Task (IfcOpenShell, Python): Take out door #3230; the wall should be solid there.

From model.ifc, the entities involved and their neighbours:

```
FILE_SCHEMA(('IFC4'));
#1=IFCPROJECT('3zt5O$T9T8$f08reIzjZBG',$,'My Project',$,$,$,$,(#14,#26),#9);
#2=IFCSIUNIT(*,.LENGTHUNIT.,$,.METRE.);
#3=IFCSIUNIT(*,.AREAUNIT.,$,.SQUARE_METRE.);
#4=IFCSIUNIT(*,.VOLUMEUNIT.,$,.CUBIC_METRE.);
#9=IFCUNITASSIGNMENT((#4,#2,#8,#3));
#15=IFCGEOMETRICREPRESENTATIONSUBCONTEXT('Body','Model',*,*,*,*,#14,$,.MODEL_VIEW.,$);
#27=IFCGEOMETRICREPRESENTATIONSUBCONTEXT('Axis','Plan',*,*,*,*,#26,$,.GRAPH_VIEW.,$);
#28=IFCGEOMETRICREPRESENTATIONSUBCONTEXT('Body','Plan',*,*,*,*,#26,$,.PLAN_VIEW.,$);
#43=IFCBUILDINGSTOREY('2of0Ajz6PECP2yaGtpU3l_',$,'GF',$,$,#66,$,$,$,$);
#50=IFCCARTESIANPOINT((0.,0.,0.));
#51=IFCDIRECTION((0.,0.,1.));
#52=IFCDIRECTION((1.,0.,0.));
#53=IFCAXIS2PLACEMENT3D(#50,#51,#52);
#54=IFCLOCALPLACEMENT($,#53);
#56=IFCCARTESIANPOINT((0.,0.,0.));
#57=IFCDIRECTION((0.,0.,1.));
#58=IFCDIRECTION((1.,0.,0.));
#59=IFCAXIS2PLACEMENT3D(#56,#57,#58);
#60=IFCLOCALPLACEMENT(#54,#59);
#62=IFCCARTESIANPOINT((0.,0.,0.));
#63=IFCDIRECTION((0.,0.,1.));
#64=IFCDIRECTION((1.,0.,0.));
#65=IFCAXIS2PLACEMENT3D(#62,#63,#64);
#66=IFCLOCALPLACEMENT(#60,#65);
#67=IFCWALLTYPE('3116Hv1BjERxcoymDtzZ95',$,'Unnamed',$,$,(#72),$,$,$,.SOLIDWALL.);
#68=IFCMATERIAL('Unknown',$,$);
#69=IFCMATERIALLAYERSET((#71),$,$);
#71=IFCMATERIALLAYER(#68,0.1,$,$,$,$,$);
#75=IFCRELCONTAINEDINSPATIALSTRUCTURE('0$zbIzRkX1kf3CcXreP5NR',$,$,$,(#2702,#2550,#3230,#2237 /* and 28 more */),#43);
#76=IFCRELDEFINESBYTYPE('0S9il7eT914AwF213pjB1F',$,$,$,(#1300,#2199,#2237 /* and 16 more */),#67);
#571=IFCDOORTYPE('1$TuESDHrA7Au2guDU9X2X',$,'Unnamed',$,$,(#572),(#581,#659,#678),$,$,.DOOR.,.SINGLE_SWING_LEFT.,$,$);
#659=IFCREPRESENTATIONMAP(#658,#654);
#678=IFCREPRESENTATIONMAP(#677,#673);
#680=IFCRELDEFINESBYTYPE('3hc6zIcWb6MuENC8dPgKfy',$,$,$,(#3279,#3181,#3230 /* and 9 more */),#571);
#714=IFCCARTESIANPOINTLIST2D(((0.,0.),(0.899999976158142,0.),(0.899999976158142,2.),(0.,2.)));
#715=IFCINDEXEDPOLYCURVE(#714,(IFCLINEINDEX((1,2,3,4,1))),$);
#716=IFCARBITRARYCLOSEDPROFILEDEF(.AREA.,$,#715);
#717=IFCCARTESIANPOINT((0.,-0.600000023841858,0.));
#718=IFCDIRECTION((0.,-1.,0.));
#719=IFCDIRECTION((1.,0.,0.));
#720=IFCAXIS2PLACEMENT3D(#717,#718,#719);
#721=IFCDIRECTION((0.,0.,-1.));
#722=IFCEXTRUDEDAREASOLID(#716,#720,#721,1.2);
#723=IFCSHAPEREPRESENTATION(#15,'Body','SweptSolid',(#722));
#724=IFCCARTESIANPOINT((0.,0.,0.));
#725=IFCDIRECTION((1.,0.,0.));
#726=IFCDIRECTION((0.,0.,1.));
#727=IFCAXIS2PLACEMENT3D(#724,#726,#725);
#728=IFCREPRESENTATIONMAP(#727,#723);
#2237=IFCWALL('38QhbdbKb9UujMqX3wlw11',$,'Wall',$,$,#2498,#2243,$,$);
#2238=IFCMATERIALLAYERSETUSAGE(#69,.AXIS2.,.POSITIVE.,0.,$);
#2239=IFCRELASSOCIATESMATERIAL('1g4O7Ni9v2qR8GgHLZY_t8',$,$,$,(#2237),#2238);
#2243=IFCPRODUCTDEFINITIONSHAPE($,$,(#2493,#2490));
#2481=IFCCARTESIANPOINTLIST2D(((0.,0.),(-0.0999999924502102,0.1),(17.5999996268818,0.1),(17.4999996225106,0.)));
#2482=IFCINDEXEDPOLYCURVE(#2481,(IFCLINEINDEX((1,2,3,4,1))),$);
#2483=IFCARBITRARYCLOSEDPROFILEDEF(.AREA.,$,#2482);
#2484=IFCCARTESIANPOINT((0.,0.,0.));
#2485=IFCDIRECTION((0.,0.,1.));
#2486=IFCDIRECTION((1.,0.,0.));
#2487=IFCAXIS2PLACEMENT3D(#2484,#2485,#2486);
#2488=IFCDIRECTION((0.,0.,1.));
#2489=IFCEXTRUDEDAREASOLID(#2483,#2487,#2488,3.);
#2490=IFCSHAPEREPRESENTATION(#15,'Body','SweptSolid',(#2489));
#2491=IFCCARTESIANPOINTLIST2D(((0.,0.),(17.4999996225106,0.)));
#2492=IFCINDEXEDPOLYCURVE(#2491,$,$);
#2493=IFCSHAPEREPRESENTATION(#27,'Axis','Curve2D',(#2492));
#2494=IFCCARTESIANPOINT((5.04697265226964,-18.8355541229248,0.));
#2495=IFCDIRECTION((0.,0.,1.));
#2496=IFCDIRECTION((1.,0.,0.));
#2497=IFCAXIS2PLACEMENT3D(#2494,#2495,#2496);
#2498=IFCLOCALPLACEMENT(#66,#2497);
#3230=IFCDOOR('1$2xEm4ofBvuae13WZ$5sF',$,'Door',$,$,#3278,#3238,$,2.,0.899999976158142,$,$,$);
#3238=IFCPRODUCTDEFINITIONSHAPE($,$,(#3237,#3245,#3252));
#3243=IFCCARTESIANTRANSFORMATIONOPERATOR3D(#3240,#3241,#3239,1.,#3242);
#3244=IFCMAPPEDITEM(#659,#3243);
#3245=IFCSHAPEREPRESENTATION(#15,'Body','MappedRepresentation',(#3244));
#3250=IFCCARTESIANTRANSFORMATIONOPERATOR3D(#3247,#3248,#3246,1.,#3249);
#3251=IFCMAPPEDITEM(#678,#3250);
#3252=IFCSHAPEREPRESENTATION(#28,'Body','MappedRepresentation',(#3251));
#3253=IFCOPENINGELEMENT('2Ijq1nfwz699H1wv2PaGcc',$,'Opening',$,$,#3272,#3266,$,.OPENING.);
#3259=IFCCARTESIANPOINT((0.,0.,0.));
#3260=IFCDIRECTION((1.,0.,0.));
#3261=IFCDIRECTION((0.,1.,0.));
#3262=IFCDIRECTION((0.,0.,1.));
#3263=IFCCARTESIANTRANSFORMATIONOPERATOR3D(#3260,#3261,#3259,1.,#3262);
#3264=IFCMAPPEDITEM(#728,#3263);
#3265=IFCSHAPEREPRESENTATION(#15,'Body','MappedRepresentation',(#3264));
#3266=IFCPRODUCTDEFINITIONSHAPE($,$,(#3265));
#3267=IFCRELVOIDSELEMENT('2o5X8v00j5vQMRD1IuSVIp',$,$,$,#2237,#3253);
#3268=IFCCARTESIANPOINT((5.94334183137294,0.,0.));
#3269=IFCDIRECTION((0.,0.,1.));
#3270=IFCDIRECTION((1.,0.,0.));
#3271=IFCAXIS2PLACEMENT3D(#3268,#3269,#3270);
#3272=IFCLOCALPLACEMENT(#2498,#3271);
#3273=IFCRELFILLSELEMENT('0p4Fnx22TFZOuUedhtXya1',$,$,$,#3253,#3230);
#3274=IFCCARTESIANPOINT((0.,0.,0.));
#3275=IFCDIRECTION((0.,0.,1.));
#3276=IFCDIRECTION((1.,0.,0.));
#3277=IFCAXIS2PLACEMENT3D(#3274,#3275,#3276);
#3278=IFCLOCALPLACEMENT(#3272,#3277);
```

```python
import ifcopenshell
import ifcopenshell.api.feature
import ifcopenshell.api.root
import ifcopenshell.geom
import ifcopenshell.util.shape

model = ifcopenshell.open("model.ifc")
settings = ifcopenshell.geom.settings()


def volume(element):
    """Net volume in cubic metres, openings subtracted."""
    shape = ifcopenshell.geom.create_shape(settings, element)
    return ifcopenshell.util.shape.get_volume(shape.geometry)


door = model.by_guid("1$2xEm4ofBvuae13WZ$5sF")
opening = door.FillsVoids[0].RelatingOpeningElement
wall = opening.VoidsElements[0].RelatingBuildingElement
before = volume(wall)

ifcopenshell.api.root.remove_product(model, product=door)
ifcopenshell.api.feature.remove_feature(model, feature=opening)

after = volume(wall)

print(f"wall volume {before:.3f} -> {after:.3f} m3")

model.write("model_rev.ifc")
```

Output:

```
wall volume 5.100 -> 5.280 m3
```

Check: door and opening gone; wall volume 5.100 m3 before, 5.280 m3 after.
